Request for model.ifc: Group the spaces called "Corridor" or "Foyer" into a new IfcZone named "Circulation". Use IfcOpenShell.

First a look at what the model holds.

```python
import ifcopenshell

model = ifcopenshell.open("model.ifc")
print(model.schema)
seen = {}
for space in model.by_type("IfcSpace"):
    seen[space.LongName] = seen.get(space.LongName, 0) + 1
for name, count in sorted(seen.items(), key=str):
    print(count, "x", name)
print("zones:", [z.Name for z in model.by_type("IfcZone")][:20])
```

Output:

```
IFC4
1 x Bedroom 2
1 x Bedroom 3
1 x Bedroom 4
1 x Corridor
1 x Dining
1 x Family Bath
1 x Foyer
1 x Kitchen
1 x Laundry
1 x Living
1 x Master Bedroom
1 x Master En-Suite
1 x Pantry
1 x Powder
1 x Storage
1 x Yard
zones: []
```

```python
import ifcopenshell
import ifcopenshell.api.group
import ifcopenshell.api.root

model = ifcopenshell.open("model.ifc")

names = {"Corridor", "Foyer"}
spaces = [s for s in model.by_type("IfcSpace") if s.LongName in names]

zone = ifcopenshell.api.root.create_entity(model, ifc_class="IfcZone", name="Circulation")
ifcopenshell.api.group.assign_group(model, products=spaces, group=zone)
print(len(spaces), "spaces in", zone.Name)

model.write("model_v2.ifc")
```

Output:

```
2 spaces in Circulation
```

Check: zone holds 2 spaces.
